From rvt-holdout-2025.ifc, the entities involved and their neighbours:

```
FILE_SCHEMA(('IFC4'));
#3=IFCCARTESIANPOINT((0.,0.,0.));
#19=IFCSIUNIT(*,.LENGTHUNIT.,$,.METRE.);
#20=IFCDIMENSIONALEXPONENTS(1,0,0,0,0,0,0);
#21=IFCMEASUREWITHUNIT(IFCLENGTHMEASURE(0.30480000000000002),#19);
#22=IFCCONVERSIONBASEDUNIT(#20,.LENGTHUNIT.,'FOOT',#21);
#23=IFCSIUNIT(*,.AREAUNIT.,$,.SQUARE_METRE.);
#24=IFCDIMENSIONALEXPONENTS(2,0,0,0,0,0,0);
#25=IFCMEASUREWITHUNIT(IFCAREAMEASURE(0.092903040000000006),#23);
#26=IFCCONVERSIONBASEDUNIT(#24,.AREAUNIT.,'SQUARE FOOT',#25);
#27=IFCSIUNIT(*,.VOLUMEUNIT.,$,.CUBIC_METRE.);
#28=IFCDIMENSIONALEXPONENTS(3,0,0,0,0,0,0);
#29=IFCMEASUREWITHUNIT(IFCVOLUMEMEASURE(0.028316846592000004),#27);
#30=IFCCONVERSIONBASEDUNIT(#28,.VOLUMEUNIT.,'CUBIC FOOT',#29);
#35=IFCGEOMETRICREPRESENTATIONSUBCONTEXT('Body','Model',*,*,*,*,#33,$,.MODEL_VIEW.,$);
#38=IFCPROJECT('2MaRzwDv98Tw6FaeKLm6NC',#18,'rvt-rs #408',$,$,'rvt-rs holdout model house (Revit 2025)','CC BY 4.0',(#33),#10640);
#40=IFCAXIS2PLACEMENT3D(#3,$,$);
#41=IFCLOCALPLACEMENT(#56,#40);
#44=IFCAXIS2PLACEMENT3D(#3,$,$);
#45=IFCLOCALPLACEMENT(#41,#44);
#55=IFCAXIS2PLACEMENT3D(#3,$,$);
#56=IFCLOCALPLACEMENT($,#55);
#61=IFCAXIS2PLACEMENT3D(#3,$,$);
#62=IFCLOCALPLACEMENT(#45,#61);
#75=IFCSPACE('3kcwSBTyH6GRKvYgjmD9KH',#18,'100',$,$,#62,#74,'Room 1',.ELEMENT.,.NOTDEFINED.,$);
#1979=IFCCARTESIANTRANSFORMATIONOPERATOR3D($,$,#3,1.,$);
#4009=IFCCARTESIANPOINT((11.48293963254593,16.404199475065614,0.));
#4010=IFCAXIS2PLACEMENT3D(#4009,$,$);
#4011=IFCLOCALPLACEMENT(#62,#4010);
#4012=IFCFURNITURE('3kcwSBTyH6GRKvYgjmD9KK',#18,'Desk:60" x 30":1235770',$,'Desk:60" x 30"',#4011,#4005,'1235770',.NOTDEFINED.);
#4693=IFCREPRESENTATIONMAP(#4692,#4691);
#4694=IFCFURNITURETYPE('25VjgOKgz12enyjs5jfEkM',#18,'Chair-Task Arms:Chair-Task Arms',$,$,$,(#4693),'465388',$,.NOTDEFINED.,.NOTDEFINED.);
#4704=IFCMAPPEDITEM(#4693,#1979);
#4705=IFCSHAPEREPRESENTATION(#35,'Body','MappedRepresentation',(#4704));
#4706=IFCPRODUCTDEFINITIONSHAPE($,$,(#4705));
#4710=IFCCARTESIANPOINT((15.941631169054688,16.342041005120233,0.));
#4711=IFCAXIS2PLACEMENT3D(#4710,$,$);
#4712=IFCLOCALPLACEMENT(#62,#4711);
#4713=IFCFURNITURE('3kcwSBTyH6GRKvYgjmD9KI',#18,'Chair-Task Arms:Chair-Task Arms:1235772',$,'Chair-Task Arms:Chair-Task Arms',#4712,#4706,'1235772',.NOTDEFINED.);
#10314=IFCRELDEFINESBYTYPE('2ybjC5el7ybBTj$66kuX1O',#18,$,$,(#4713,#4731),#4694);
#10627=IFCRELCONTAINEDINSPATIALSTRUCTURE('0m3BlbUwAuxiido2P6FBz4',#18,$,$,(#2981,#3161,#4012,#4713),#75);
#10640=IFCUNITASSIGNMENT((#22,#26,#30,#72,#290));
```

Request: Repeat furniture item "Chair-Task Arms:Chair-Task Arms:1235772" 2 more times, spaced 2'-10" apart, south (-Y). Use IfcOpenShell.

```python
import numpy as np
import ifcopenshell
import ifcopenshell.api.geometry
import ifcopenshell.api.root
import ifcopenshell.util.element
import ifcopenshell.util.placement
import ifcopenshell.util.unit

model = ifcopenshell.open("rvt-holdout-2025.ifc")
unit_scale = ifcopenshell.util.unit.calculate_unit_scale(model)


def reuse_history(source, copy):
    """copy_class also copies each property set's owner history, people and application; keep the originals."""
    for rel in copy.IsDefinedBy:
        if rel.is_a("IfcRelDefinesByProperties") and (history := rel.RelatingPropertyDefinition.OwnerHistory):
            rel.RelatingPropertyDefinition.OwnerHistory = source.OwnerHistory
            ifcopenshell.util.element.remove_deep2(model, history)


source = model.by_guid("3kcwSBTyH6GRKvYgjmD9KI")
base = ifcopenshell.util.placement.get_local_placement(source.ObjectPlacement)
step = np.array([0.0, -1.0, 0.0]) * 34 * 0.0254 / unit_scale

for i in range(1, 3):
    copy = ifcopenshell.api.root.copy_class(model, product=source)
    copy.Representation = ifcopenshell.util.element.copy_deep(
        model, source.Representation, exclude=["IfcGeometricRepresentationContext", "IfcRepresentationMap"]
    )
    copy.Name = "Chair-Task Arms:Chair-Task Arms"
    copy.Tag = None
    reuse_history(source, copy)
    matrix = base.copy()
    matrix[:3, 3] += i * step
    print("added at", matrix[:3, 3].round(3) + 0.0)
    ifcopenshell.api.geometry.edit_object_placement(model, product=copy, matrix=matrix, is_si=False)

model.write("rvt-holdout-2025_updated.ifc")
```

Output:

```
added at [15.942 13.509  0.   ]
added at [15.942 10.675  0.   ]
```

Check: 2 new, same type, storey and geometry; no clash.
